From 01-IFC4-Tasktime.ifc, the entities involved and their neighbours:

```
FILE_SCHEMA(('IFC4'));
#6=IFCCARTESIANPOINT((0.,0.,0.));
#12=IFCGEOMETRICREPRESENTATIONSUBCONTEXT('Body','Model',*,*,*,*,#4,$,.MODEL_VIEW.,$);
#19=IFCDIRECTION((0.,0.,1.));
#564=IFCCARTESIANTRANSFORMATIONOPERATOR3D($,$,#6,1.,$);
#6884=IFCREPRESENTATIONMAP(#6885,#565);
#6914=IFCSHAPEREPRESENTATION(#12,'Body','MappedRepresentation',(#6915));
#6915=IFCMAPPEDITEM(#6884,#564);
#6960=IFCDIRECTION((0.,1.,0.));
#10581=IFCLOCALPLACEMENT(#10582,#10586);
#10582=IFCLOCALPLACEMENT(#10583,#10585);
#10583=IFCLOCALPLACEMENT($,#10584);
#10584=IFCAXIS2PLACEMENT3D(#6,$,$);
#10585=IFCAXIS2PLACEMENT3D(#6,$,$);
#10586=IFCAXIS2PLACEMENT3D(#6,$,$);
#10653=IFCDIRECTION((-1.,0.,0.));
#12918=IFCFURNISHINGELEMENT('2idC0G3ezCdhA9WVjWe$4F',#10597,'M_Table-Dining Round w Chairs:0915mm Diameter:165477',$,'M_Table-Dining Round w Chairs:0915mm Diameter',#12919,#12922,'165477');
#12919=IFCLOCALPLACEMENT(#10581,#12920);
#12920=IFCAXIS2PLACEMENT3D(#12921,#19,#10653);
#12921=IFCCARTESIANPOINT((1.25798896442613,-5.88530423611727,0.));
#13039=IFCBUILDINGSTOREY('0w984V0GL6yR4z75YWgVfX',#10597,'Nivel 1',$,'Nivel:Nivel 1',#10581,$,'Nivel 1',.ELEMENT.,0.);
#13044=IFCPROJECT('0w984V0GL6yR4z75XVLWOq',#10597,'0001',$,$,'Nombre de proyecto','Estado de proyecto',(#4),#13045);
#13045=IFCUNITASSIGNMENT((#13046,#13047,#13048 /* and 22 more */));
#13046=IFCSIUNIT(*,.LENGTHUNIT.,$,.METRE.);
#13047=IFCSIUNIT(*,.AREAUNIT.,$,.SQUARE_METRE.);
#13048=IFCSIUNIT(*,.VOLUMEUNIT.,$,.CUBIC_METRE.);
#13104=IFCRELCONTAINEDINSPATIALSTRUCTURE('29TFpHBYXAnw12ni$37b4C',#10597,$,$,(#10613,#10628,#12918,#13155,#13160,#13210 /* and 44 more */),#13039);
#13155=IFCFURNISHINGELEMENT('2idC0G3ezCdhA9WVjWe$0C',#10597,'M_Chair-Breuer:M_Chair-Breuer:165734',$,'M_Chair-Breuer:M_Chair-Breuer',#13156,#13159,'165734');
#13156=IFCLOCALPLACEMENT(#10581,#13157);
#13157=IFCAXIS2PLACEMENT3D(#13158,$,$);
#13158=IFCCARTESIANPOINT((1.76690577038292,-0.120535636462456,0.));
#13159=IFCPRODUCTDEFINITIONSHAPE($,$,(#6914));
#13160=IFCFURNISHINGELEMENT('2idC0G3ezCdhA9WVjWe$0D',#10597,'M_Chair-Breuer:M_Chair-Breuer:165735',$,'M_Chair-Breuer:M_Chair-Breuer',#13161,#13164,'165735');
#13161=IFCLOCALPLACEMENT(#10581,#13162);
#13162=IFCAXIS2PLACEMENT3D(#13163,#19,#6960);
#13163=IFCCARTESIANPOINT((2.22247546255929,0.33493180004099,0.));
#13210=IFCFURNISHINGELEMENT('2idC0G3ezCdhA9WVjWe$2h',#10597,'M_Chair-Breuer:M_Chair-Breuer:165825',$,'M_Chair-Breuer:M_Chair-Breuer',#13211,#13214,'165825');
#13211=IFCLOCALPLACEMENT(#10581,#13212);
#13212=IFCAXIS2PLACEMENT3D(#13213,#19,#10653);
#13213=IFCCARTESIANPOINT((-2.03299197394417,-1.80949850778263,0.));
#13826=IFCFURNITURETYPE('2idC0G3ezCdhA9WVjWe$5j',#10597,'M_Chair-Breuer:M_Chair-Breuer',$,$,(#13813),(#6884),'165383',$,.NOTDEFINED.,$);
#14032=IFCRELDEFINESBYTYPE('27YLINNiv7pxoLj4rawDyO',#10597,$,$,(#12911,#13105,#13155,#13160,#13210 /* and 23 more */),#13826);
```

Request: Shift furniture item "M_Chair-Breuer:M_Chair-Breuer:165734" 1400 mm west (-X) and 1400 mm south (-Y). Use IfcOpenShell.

```python
import ifcopenshell
import ifcopenshell.api.geometry
import ifcopenshell.util.placement
import ifcopenshell.util.unit

model = ifcopenshell.open("01-IFC4-Tasktime.ifc")
unit_scale = ifcopenshell.util.unit.calculate_unit_scale(model)

item = model.by_id(13155)
matrix = ifcopenshell.util.placement.get_local_placement(item.ObjectPlacement)
matrix[0, 3] -= 1.4 / unit_scale
matrix[1, 3] -= 1.4 / unit_scale
ifcopenshell.api.geometry.edit_object_placement(model, product=item, matrix=matrix, is_si=False)

print(ifcopenshell.util.placement.get_local_placement(item.ObjectPlacement).round(3) + 0.0)

model.write("01-IFC4-Tasktime_edited.ifc")
```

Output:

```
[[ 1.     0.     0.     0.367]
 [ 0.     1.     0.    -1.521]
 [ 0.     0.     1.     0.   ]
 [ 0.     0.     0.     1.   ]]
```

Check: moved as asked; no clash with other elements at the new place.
